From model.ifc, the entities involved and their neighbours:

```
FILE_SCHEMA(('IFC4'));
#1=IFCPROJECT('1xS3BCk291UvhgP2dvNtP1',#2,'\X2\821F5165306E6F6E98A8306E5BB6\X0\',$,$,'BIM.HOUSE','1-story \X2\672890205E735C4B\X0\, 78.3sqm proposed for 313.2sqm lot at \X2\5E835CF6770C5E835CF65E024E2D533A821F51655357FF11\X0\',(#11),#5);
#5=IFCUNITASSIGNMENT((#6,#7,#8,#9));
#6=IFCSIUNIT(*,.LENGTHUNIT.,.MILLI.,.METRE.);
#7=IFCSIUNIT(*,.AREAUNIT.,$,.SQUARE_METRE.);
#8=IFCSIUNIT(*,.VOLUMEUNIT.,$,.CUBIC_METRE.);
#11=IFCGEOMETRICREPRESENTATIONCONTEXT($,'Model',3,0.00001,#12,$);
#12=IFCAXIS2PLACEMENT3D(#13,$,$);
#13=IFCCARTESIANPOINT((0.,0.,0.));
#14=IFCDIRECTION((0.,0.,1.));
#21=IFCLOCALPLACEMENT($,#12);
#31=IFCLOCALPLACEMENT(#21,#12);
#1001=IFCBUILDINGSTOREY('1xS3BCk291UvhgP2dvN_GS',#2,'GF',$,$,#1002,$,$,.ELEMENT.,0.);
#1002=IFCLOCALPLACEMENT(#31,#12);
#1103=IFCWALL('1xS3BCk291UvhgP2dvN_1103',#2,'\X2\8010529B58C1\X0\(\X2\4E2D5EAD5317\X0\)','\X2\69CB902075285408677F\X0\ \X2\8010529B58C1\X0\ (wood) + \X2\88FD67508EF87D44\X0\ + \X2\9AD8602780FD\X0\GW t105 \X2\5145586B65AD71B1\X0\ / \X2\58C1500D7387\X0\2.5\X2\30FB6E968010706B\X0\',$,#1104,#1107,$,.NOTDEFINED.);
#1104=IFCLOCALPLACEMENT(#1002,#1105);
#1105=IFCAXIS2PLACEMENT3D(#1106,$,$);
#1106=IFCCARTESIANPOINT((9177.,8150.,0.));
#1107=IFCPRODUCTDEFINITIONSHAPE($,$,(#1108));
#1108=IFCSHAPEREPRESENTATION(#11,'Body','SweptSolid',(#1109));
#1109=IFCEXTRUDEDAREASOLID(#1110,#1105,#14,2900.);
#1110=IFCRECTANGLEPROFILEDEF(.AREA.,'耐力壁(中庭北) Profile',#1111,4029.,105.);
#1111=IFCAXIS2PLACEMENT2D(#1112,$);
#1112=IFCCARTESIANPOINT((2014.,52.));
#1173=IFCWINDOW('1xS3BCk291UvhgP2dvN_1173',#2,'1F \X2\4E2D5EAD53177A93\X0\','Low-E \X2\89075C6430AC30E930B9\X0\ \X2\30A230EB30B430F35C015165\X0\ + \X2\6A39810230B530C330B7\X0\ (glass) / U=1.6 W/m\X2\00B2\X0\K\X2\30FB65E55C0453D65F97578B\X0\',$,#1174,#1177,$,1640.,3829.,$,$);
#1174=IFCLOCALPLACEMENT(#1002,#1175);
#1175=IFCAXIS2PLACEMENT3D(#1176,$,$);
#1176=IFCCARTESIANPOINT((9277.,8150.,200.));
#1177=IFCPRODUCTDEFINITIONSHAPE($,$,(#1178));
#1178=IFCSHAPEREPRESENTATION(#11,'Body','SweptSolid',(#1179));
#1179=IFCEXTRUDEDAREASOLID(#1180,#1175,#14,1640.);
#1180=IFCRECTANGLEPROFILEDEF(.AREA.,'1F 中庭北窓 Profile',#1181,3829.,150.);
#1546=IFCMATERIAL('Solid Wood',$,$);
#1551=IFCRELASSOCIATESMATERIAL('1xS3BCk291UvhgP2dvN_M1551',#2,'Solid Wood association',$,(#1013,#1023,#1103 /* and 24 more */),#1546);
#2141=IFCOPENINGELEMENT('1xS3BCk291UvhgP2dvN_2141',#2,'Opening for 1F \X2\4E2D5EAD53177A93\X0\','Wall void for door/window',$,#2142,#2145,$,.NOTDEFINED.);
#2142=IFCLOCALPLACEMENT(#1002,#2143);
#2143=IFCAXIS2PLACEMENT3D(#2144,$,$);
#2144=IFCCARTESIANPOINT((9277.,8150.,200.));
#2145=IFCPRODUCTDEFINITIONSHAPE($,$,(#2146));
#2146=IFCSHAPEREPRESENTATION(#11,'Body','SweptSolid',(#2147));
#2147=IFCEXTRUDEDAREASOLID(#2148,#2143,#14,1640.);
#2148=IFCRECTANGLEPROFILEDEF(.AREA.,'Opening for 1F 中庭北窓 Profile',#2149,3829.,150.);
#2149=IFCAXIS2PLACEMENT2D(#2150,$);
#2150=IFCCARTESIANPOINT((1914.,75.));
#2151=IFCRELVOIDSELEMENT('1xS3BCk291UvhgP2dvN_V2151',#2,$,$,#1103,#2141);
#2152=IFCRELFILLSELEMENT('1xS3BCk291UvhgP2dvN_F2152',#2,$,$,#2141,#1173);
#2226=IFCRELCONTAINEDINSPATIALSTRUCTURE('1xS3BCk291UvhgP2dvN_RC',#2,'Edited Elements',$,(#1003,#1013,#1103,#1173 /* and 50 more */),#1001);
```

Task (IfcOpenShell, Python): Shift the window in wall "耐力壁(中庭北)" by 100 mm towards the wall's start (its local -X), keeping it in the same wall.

```python
import ifcopenshell
import ifcopenshell.api.geometry
import ifcopenshell.util.placement

model = ifcopenshell.open("model.ifc")

window = model.by_guid("1xS3BCk291UvhgP2dvN_1173")
opening = window.FillsVoids[0].RelatingOpeningElement
wall = opening.VoidsElements[0].RelatingBuildingElement

wall_matrix = ifcopenshell.util.placement.get_local_placement(wall.ObjectPlacement)
shift = wall_matrix[:3, 0] * -100.0
before = ifcopenshell.util.placement.get_local_placement(window.ObjectPlacement)[:3, 3].copy()

# The window is not placed relative to its opening, so move both.
for product in (opening, window):
    matrix = ifcopenshell.util.placement.get_local_placement(product.ObjectPlacement)
    matrix[:3, 3] += shift
    ifcopenshell.api.geometry.edit_object_placement(model, product=product, matrix=matrix, is_si=False)

after = ifcopenshell.util.placement.get_local_placement(window.ObjectPlacement)[:3, 3]
print("window moved by", (after - before).round(3) + 0.0)

model.write("model_v2.ifc")
```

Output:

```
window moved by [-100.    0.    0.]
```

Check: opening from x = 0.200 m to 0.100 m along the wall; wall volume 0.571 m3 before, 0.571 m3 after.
